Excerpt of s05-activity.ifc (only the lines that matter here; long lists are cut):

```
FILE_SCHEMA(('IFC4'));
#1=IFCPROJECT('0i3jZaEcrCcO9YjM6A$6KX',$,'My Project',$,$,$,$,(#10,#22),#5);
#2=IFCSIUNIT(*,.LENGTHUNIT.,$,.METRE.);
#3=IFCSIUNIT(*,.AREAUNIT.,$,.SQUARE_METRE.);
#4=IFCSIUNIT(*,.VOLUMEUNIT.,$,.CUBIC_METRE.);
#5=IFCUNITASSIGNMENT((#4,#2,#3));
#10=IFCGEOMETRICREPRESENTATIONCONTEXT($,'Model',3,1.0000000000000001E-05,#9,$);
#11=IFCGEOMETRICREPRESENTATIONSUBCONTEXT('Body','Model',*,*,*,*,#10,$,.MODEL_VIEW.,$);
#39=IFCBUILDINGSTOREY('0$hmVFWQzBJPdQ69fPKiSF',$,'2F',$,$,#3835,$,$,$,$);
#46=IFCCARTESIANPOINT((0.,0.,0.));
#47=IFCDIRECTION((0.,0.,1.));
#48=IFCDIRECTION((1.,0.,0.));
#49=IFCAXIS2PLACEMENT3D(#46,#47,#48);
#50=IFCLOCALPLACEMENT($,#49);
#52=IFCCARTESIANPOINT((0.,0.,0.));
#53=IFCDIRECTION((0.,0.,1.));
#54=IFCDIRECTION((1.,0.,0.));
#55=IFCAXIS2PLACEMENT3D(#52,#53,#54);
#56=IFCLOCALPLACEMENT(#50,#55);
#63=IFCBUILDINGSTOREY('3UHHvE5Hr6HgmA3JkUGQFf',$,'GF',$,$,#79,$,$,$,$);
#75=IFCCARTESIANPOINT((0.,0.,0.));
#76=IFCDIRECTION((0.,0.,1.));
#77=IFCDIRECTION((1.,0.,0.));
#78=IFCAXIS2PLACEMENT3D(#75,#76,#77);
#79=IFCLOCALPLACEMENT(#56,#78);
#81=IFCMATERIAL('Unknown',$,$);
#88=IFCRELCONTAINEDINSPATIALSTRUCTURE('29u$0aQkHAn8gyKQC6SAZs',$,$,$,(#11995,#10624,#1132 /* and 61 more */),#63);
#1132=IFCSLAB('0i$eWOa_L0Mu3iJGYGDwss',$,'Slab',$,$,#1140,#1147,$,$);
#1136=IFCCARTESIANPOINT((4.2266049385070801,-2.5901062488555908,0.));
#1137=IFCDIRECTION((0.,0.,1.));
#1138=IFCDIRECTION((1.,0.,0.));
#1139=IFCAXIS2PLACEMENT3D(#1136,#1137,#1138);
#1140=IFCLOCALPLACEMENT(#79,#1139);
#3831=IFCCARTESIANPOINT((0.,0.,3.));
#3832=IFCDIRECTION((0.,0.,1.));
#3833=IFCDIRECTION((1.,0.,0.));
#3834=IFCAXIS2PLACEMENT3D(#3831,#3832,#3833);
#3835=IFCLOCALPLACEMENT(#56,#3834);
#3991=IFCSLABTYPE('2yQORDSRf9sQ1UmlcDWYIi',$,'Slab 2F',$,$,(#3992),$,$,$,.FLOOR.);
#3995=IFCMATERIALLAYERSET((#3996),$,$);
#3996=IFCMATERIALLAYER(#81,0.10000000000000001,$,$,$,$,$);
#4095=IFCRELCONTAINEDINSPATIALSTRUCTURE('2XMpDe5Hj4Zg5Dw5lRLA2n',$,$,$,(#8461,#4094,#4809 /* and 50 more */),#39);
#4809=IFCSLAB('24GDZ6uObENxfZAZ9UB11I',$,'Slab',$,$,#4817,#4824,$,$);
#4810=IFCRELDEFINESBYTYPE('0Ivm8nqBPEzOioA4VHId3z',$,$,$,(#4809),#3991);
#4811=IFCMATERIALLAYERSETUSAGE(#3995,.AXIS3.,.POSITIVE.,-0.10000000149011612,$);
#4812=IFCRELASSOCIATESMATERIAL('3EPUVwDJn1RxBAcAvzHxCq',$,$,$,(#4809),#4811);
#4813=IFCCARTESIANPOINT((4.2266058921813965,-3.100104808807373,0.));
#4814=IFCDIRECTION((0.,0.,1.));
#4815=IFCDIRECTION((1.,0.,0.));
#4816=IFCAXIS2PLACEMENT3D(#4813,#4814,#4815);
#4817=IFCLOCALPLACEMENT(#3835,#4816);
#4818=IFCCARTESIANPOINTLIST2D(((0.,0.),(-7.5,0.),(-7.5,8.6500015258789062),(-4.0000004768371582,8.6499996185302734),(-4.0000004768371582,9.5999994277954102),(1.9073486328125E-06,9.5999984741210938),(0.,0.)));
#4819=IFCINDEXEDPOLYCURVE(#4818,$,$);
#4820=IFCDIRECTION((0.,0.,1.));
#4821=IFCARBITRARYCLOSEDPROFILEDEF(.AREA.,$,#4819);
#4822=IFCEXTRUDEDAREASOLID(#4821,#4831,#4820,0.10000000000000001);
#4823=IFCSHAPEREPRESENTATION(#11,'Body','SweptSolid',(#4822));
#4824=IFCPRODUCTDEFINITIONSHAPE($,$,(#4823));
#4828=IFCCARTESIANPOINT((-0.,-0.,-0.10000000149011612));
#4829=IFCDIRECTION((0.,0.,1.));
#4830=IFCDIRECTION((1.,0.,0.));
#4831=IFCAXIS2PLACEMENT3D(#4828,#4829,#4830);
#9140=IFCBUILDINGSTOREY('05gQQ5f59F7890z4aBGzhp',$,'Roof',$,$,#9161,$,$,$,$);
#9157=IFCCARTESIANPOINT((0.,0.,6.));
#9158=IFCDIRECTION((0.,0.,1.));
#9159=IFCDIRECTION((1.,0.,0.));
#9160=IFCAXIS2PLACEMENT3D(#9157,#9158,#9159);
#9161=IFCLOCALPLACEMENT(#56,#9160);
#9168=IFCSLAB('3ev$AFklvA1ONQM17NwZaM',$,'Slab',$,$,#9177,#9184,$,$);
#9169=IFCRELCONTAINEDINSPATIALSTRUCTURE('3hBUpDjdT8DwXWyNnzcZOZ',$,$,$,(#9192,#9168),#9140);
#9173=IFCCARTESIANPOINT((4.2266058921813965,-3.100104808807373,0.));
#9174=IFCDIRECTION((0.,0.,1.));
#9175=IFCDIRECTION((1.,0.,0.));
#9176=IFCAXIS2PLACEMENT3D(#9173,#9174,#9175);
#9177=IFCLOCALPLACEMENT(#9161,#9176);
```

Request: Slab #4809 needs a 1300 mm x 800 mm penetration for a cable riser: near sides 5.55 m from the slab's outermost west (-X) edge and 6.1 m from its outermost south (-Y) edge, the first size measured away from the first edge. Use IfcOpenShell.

```python
import numpy as np
import ifcopenshell
import ifcopenshell.api.feature
import ifcopenshell.api.geometry
import ifcopenshell.api.root
import ifcopenshell.geom
import ifcopenshell.util.placement
import ifcopenshell.util.representation
import ifcopenshell.util.shape
import ifcopenshell.util.unit

model = ifcopenshell.open("s05-activity.ifc")
unit_scale = ifcopenshell.util.unit.calculate_unit_scale(model)
settings = ifcopenshell.geom.settings()


def volume(element):
    """Net volume in cubic metres, openings subtracted."""
    shape = ifcopenshell.geom.create_shape(settings, element)
    return ifcopenshell.util.shape.get_volume(shape.geometry)


slab = model.by_id(4809)
before = volume(slab)

# Extent in the slab's own axes, in metres. The edges named are its -X and -Y sides.
slab_shape = ifcopenshell.geom.create_shape(settings, slab)
vertices = ifcopenshell.util.shape.get_vertices(slab_shape.geometry)
x_min, y_min, bottom = vertices.min(axis=0)
top = vertices[:, 2].max()

opening = ifcopenshell.api.root.create_entity(model, ifc_class="IfcOpeningElement", name="Cable riser opening", predefined_type="OPENING")
context = ifcopenshell.util.representation.get_context(model, "Model", "Body", "MODEL_VIEW")
width, depth = 1.3, 0.8
outline = [(0.0, 0.0), (width, 0.0), (width, depth), (0.0, depth), (0.0, 0.0)]
# Overshoot both faces by 50 mm so the cut is clean.
shape = ifcopenshell.api.geometry.add_slab_representation(
    model, context=context, depth=top - bottom + 0.1, polyline=outline
)
ifcopenshell.api.geometry.assign_representation(model, product=opening, representation=shape)

matrix = ifcopenshell.util.placement.get_local_placement(slab.ObjectPlacement)
matrix[:, 3] = matrix @ np.append(np.array([x_min + 5.55, y_min + 6.1, bottom - 0.05]) / unit_scale, 1.0)
ifcopenshell.api.geometry.edit_object_placement(model, product=opening, matrix=matrix, is_si=False)
ifcopenshell.api.feature.add_feature(model, feature=opening, element=slab)

after = volume(slab)

print(f"slab volume {before:.3f} -> {after:.3f} m3")

model.write("s05-activity_rev.ifc")
```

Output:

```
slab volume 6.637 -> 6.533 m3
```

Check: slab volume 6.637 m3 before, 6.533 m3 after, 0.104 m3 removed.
